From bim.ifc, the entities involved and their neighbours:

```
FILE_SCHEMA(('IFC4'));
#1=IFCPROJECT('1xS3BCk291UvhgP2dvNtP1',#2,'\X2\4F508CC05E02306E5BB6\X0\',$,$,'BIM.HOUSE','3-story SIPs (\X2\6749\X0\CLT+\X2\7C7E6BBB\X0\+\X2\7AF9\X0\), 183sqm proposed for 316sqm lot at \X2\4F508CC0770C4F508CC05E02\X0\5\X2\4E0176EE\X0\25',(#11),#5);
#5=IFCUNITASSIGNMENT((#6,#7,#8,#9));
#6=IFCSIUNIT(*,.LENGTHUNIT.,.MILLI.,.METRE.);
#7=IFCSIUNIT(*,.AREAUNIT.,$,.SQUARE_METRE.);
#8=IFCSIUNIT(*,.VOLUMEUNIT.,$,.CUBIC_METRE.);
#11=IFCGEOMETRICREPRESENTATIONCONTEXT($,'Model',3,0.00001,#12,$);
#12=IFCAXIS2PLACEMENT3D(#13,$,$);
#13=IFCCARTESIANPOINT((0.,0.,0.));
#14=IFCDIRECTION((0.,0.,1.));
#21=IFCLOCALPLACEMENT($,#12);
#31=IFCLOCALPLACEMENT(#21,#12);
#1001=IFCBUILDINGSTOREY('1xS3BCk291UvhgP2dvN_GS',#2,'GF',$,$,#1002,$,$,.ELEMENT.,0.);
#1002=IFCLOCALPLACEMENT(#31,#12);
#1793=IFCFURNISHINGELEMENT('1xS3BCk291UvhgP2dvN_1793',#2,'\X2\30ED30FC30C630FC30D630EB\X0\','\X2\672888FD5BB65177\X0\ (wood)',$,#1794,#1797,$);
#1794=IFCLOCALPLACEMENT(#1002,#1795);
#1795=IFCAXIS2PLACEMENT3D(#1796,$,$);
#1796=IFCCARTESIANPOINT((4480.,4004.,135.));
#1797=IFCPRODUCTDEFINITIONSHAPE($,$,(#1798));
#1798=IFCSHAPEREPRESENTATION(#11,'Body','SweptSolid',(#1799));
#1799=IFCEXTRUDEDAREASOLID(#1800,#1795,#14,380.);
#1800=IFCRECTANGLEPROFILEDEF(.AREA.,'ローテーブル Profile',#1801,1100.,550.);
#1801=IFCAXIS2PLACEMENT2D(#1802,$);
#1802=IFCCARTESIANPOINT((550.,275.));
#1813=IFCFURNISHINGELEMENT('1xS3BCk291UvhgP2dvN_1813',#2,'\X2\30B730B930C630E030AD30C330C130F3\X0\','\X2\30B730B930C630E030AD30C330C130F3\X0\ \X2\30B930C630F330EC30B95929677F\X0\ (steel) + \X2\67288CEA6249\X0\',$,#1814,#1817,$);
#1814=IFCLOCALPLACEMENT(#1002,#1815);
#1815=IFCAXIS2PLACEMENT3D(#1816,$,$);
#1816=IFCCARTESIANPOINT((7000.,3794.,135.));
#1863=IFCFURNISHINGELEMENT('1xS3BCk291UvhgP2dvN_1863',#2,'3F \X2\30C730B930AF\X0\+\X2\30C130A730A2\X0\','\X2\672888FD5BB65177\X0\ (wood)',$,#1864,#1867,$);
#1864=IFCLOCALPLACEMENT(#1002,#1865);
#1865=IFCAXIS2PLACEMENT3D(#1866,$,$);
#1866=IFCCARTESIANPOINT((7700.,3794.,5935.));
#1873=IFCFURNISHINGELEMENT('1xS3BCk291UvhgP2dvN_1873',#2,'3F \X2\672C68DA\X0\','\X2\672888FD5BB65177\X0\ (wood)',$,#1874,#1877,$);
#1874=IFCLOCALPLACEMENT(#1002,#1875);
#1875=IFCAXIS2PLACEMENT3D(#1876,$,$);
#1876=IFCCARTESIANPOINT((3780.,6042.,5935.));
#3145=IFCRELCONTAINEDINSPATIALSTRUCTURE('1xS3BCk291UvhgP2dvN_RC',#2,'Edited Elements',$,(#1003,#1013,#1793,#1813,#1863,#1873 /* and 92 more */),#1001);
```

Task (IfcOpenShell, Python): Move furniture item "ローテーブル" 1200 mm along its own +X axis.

```python
import ifcopenshell
import ifcopenshell.api.geometry
import ifcopenshell.util.placement

model = ifcopenshell.open("bim.ifc")

item = model.by_guid("1xS3BCk291UvhgP2dvN_1793")
matrix = ifcopenshell.util.placement.get_local_placement(item.ObjectPlacement)
matrix[:3, 3] += matrix[:3, 0] * 1200.0
ifcopenshell.api.geometry.edit_object_placement(model, product=item, matrix=matrix, is_si=False)

print(ifcopenshell.util.placement.get_local_placement(item.ObjectPlacement).round(3) + 0.0)

model.write("bim_rev.ifc")
```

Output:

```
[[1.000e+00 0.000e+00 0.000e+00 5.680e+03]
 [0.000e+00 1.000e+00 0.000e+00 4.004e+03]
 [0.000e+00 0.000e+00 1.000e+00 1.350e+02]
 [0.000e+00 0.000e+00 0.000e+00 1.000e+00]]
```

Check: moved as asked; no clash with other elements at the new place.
